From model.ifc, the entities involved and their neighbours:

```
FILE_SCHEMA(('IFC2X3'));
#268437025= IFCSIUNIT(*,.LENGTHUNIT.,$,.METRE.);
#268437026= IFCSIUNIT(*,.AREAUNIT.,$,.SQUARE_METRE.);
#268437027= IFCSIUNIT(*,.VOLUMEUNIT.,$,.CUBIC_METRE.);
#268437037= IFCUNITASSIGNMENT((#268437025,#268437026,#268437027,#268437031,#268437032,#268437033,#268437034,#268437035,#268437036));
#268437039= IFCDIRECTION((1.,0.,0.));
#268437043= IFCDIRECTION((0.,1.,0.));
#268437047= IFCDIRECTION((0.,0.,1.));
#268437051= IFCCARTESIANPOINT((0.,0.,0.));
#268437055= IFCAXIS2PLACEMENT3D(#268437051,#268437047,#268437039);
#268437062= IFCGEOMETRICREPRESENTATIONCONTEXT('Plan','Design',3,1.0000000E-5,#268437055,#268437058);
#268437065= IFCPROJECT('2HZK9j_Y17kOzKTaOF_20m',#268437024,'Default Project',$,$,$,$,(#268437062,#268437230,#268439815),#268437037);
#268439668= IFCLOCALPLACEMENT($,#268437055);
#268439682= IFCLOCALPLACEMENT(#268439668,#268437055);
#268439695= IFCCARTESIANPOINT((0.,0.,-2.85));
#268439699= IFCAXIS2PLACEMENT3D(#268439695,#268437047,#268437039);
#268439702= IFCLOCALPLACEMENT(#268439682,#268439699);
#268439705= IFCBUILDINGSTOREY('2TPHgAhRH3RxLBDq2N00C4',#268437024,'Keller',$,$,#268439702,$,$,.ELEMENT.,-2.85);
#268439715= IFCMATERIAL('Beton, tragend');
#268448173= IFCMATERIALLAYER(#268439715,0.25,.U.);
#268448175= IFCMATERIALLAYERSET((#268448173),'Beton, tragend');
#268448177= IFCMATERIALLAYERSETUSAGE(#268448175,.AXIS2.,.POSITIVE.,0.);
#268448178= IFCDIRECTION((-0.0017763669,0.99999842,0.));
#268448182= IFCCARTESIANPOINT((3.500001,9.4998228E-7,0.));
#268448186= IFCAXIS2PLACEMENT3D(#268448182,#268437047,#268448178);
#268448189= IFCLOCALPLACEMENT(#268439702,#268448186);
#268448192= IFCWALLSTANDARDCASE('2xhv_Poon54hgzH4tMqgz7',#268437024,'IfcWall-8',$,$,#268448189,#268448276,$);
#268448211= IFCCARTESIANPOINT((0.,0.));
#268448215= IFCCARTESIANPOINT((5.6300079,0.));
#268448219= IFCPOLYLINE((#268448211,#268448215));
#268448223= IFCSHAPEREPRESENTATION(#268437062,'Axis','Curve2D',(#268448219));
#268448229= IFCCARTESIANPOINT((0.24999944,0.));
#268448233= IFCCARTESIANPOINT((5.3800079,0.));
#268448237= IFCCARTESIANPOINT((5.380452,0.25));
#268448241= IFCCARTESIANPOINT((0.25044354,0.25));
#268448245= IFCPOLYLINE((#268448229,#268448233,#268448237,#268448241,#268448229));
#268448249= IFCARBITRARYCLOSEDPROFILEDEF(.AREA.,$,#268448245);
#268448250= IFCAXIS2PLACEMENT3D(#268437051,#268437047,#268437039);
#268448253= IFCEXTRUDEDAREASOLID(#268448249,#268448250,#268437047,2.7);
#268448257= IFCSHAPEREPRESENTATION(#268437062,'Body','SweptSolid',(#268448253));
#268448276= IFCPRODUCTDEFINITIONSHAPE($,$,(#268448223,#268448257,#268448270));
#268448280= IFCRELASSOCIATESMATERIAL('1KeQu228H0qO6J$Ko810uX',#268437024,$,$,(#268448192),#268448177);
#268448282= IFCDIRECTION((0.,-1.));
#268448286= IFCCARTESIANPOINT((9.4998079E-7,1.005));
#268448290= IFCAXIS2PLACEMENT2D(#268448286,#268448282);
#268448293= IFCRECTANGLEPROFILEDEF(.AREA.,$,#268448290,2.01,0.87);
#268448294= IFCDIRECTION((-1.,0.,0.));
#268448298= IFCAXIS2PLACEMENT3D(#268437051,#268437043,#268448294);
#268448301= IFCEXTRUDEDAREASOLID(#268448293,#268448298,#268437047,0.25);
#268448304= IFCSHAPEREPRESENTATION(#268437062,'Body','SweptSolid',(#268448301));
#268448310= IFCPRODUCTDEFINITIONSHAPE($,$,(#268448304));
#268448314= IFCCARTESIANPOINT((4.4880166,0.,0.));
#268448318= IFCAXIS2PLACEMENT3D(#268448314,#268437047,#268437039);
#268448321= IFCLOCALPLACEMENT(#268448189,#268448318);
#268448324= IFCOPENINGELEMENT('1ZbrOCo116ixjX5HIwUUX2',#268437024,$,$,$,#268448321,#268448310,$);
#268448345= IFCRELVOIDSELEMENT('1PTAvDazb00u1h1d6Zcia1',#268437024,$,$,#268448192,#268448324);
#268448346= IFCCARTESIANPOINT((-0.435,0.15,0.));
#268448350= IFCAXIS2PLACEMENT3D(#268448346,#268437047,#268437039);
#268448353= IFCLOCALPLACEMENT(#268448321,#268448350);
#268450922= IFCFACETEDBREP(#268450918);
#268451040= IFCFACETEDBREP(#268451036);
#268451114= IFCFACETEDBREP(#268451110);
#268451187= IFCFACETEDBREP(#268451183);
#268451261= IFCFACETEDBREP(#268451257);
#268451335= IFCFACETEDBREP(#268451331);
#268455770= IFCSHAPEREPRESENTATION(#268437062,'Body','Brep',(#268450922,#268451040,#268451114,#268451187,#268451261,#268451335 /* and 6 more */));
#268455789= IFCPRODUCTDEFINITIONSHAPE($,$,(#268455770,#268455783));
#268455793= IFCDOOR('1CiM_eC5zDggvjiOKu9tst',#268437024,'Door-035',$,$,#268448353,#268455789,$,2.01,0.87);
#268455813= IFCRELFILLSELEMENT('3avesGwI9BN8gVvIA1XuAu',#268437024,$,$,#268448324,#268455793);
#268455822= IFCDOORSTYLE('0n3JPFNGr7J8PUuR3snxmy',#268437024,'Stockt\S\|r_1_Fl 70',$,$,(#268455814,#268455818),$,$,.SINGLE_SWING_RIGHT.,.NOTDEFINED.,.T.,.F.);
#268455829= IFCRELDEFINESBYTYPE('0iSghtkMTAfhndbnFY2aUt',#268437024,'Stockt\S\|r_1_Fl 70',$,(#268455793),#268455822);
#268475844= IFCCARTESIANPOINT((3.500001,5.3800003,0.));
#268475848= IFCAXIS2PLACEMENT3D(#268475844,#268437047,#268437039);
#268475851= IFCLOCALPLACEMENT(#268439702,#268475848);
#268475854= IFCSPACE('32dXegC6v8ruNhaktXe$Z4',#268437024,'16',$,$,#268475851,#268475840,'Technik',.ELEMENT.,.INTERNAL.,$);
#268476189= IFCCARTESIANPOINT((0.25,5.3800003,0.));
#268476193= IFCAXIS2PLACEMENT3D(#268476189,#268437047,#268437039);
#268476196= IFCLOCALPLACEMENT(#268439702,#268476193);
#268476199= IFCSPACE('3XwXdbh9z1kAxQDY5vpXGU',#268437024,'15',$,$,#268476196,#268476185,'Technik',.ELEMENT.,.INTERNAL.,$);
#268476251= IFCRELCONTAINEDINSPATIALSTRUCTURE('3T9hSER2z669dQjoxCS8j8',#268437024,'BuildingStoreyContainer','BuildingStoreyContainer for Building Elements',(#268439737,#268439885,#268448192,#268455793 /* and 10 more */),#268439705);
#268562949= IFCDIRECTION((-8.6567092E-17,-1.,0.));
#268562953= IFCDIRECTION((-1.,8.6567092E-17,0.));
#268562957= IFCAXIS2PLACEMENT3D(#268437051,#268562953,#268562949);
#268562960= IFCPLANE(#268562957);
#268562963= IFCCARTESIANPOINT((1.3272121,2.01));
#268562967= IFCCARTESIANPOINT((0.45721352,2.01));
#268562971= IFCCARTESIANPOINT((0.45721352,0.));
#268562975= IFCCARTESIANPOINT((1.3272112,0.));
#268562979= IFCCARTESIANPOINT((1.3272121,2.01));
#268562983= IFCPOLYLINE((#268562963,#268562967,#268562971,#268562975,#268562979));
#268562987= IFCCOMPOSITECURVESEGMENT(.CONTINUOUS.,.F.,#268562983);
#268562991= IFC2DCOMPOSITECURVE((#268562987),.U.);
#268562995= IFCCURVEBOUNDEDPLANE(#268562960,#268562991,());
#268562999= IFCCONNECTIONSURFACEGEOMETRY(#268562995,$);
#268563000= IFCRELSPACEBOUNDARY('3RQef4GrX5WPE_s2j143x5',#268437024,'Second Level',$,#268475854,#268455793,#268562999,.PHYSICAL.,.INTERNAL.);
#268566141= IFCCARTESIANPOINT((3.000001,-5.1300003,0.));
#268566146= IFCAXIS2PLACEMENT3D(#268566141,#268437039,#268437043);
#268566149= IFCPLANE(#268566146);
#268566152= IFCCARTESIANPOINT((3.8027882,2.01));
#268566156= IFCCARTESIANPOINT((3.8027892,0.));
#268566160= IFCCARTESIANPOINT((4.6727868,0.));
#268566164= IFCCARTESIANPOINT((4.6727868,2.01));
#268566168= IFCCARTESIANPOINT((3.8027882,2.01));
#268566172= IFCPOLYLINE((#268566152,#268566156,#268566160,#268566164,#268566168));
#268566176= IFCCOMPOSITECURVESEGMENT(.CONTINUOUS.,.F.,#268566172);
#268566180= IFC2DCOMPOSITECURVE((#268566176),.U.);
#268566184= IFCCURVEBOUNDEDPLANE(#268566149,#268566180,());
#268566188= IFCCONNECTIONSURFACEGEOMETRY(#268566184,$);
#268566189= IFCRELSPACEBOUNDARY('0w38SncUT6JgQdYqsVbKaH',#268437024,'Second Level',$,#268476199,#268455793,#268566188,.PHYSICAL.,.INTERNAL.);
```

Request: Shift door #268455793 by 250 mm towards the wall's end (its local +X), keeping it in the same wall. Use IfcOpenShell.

```python
import numpy as np
import ifcopenshell
import ifcopenshell.api.geometry
import ifcopenshell.util.placement

model = ifcopenshell.open("model.ifc")

door = model.by_id(268455793)
opening = door.FillsVoids[0].RelatingOpeningElement
wall = opening.VoidsElements[0].RelatingBuildingElement

wall_matrix = ifcopenshell.util.placement.get_local_placement(wall.ObjectPlacement)
shift = wall_matrix[:3, 0] * 0.25
before = ifcopenshell.util.placement.get_local_placement(door.ObjectPlacement)[:3, 3].copy()

# The door is placed relative to its opening, so it follows when the opening moves.
matrix = ifcopenshell.util.placement.get_local_placement(opening.ObjectPlacement)
matrix[:3, 3] += shift
ifcopenshell.api.geometry.edit_object_placement(
    model, product=opening, matrix=matrix, is_si=False, should_transform_children=True
)

# Space boundary surfaces are stored in each space's coordinates; move them too.
for rel in door.ProvidesBoundaries:
    if not rel.ConnectionGeometry:
        continue
    surface = rel.ConnectionGeometry.SurfaceOnRelatingElement.BasisSurface
    space_matrix = ifcopenshell.util.placement.get_local_placement(rel.RelatingSpace.ObjectPlacement)
    point = np.array(surface.Position.Location.Coordinates) + space_matrix[:3, :3].T @ shift
    surface.Position = model.createIfcAxis2Placement3D(
        model.createIfcCartesianPoint(point.tolist()), surface.Position.Axis, surface.Position.RefDirection
    )

after = ifcopenshell.util.placement.get_local_placement(door.ObjectPlacement)[:3, 3]
print("door moved by", (after - before).round(3) + 0.0)

model.write("model_v2.ifc")
```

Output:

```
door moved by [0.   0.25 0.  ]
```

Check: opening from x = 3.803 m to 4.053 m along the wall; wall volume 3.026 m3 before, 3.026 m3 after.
